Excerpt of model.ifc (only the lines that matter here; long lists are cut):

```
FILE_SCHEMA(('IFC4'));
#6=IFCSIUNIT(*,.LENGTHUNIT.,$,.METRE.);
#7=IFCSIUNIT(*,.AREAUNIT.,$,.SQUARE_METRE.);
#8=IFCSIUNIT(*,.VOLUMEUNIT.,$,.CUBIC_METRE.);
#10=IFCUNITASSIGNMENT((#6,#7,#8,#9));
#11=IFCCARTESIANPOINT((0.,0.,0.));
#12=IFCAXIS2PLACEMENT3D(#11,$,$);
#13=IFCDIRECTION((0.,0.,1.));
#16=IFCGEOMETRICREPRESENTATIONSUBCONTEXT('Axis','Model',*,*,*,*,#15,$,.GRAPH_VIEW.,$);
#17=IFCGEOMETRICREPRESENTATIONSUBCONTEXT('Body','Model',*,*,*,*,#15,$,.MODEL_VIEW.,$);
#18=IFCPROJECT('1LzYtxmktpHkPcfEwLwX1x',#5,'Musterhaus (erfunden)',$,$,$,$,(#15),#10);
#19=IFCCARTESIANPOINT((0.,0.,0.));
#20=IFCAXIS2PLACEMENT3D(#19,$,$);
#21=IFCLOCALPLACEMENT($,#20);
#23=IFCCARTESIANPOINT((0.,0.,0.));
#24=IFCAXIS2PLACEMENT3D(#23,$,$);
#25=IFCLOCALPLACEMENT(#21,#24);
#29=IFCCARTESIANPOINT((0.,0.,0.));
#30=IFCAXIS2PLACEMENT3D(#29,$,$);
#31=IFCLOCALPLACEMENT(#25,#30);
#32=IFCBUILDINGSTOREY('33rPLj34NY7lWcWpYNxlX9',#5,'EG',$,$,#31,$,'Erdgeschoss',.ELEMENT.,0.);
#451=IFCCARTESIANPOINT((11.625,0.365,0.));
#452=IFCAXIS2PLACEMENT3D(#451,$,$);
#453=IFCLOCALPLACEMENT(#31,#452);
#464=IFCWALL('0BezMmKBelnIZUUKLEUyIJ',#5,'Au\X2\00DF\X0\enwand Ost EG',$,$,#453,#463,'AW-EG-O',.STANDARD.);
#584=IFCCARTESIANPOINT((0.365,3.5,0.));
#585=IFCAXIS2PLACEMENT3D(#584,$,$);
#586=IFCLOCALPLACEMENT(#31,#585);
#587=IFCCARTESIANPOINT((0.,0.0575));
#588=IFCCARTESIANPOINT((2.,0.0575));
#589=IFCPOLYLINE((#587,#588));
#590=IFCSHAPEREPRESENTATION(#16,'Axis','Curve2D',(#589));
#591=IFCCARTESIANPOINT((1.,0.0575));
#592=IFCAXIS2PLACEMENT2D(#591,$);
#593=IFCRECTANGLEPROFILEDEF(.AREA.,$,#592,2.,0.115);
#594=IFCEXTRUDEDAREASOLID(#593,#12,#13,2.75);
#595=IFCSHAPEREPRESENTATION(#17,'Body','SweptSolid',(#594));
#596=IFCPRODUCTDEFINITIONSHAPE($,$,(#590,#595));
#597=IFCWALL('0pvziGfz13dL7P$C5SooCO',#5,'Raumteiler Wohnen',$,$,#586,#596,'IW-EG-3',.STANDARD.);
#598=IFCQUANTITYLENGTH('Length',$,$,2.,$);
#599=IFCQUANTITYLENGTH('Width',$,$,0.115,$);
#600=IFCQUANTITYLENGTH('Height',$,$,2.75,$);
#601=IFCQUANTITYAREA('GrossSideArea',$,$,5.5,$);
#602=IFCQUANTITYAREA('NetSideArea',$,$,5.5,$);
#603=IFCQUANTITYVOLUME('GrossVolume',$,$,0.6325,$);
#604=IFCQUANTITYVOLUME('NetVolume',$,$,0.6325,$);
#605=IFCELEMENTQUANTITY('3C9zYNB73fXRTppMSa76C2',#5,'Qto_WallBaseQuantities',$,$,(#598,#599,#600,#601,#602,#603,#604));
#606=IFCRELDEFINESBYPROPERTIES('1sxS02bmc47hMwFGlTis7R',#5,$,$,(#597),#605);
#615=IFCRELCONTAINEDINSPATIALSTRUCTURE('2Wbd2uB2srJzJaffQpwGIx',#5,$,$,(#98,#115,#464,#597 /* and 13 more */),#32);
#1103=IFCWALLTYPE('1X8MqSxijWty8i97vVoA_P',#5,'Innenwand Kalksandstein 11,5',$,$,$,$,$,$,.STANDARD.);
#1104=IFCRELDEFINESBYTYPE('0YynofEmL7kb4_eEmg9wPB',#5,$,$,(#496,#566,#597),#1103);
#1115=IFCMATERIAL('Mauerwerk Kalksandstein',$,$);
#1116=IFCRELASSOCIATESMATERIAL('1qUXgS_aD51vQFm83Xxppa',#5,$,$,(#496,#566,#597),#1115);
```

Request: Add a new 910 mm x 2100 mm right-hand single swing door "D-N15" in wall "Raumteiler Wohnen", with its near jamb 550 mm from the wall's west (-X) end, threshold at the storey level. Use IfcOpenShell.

```python
import numpy as np
import ifcopenshell
import ifcopenshell.api.feature
import ifcopenshell.api.geometry
import ifcopenshell.api.pset
import ifcopenshell.api.root
import ifcopenshell.api.spatial
import ifcopenshell.geom
import ifcopenshell.util.element
import ifcopenshell.util.placement
import ifcopenshell.util.representation
import ifcopenshell.util.shape
import ifcopenshell.util.unit

model = ifcopenshell.open("model.ifc")
unit_scale = ifcopenshell.util.unit.calculate_unit_scale(model)
area_scale = ifcopenshell.util.unit.calculate_unit_scale(model, "AREAUNIT")
volume_scale = ifcopenshell.util.unit.calculate_unit_scale(model, "VOLUMEUNIT")
settings = ifcopenshell.geom.settings()


def volume(element):
    """Net volume in cubic metres, openings subtracted."""
    shape = ifcopenshell.geom.create_shape(settings, element)
    return ifcopenshell.util.shape.get_volume(shape.geometry)


wall = model.by_id(597)
storey = ifcopenshell.util.element.get_container(wall, ifc_class="IfcBuildingStorey")
context = ifcopenshell.util.representation.get_context(model, "Model", "Body", "MODEL_VIEW")
before = volume(wall)

width, height, from_end, sill = 0.91, 2.1, 0.55, 0.0  # metres

# The wall runs along its own X axis, and the end named is its -X end.
wall_shape = ifcopenshell.geom.create_shape(settings, wall)
x, y, z = ifcopenshell.util.shape.get_vertices(wall_shape.geometry).T
start = x.min() + from_end
face, thickness = float(y.min()), float(y.max() - y.min())
wall_matrix = ifcopenshell.util.placement.get_local_placement(wall.ObjectPlacement)
level = ifcopenshell.util.placement.get_local_placement(storey.ObjectPlacement)[2, 3]


def in_wall(x, y):
    """Placement at x, y metres in the wall's axes, at sill height."""
    matrix = wall_matrix.copy()
    matrix[:, 3] = wall_matrix @ np.array([x / unit_scale, y / unit_scale, 0.0, 1.0])
    matrix[2, 3] = level + sill / unit_scale
    return matrix


# Opening: a box that overshoots both wall faces by 50 mm.
opening = ifcopenshell.api.root.create_entity(model, ifc_class="IfcOpeningElement", predefined_type="OPENING")
box = ifcopenshell.api.geometry.add_wall_representation(
    model, context=context, length=width, height=height, thickness=thickness + 0.1
)
ifcopenshell.api.geometry.assign_representation(model, product=opening, representation=box)
ifcopenshell.api.geometry.edit_object_placement(model, product=opening, matrix=in_wall(start, face - 0.05), is_si=False)
ifcopenshell.api.feature.add_feature(model, feature=opening, element=wall)

door = ifcopenshell.api.root.create_entity(model, ifc_class="IfcDoor", name="D-N15", predefined_type="DOOR")
door.OverallWidth, door.OverallHeight = width / unit_scale, height / unit_scale
door.OperationType = "SINGLE_SWING_RIGHT"
body = ifcopenshell.api.geometry.add_door_representation(
    model,
    context=context,
    overall_width=door.OverallWidth,
    overall_height=door.OverallHeight,
    operation_type="SINGLE_SWING_RIGHT",
    lining_properties={"LiningDepth": thickness / unit_scale, "ThresholdDepth": thickness / unit_scale},
)
ifcopenshell.api.geometry.assign_representation(model, product=door, representation=body)
ifcopenshell.api.spatial.assign_container(model, products=[door], relating_structure=storey)
ifcopenshell.api.feature.add_filling(model, opening=opening, element=door)

# The lining spans the wall, so the door starts at the wall face.
ifcopenshell.api.geometry.edit_object_placement(model, product=door, matrix=in_wall(start, face), is_si=False)

after = volume(wall)

# Update the wall's stored quantities.
qto = model.by_id(ifcopenshell.util.element.get_pset(wall, "Qto_WallBaseQuantities", should_inherit=False)["id"])
ifcopenshell.api.pset.edit_qto(model, qto=qto, properties={
    "NetSideArea": after / thickness / area_scale,
    "NetVolume": after / volume_scale,
})

print(f"wall volume {before:.3f} -> {after:.3f} m3")

model.write("model-out.ifc")
```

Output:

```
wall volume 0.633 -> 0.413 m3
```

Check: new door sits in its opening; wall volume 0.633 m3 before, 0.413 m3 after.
